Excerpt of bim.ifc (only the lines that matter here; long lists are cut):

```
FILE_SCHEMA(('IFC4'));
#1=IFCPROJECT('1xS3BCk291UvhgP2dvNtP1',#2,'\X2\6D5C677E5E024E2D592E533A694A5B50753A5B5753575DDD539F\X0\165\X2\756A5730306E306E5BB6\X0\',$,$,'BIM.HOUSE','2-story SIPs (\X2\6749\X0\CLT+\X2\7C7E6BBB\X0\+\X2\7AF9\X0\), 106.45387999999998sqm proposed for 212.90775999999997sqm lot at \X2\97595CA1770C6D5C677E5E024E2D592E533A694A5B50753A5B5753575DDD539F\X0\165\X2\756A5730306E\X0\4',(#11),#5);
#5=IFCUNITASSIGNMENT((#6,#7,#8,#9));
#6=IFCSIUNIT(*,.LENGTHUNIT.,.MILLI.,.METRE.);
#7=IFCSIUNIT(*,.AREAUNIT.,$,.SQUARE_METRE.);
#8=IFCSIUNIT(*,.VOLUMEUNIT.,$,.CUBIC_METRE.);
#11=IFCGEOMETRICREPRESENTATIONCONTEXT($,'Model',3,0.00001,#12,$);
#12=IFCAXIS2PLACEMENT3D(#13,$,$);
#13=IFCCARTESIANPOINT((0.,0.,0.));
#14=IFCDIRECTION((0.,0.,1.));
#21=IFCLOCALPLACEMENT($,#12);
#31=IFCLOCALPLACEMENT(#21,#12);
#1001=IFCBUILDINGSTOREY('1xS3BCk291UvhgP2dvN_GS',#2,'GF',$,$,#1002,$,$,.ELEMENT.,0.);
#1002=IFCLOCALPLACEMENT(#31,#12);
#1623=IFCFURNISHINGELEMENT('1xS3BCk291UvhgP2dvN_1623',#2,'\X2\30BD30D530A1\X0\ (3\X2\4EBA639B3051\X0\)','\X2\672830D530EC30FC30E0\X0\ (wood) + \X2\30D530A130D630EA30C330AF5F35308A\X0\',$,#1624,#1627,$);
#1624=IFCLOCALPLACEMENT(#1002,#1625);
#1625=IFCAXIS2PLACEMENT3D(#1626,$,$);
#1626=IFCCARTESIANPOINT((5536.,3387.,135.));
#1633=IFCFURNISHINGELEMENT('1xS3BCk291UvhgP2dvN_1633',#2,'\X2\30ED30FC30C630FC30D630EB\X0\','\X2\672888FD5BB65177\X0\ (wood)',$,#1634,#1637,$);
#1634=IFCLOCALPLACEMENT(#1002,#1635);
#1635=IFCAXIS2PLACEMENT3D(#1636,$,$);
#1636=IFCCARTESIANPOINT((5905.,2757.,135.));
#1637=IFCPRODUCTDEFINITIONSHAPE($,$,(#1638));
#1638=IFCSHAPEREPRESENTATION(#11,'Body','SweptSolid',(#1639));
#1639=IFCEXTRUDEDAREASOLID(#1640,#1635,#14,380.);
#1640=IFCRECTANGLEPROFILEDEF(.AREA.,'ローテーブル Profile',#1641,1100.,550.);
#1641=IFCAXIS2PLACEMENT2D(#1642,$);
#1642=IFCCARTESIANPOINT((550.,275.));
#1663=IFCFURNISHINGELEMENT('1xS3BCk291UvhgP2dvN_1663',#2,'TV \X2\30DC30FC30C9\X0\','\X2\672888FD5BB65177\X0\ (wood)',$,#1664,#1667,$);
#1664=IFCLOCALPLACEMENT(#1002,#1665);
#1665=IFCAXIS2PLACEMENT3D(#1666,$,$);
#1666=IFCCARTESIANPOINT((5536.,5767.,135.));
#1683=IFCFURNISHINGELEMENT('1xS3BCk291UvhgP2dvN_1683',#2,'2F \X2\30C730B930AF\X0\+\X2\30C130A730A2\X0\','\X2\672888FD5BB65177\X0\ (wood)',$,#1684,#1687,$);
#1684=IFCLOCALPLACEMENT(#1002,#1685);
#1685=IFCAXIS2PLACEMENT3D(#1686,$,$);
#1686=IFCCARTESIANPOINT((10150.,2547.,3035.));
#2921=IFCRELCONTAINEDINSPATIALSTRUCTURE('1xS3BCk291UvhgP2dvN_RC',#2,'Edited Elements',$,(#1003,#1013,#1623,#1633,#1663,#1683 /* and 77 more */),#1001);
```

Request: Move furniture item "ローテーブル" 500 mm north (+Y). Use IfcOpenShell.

```python
import ifcopenshell
import ifcopenshell.api.geometry
import ifcopenshell.util.placement

model = ifcopenshell.open("bim.ifc")

item = model.by_id(1633)
matrix = ifcopenshell.util.placement.get_local_placement(item.ObjectPlacement)
matrix[1, 3] += 500.0
ifcopenshell.api.geometry.edit_object_placement(model, product=item, matrix=matrix, is_si=False)

print(ifcopenshell.util.placement.get_local_placement(item.ObjectPlacement).round(3) + 0.0)

model.write("bim_updated.ifc")
```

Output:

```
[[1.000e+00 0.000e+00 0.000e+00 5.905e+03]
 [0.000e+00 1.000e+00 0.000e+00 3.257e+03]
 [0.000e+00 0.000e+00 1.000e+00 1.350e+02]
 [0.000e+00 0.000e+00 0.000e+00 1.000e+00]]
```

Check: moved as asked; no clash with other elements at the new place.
